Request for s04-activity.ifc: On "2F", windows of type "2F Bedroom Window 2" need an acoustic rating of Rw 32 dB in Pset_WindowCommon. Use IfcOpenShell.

First a look at what the model holds.

```python
import ifcopenshell
import ifcopenshell.util.element

model = ifcopenshell.open("s04-activity.ifc")
print(model.schema)
storey = next(s for s in model.by_type("IfcBuildingStorey") if s.Name == "2F")
windows = [e for e in ifcopenshell.util.element.get_decomposition(storey) if e.is_a("IfcWindow")]
seen = {}
for e in windows:
    element_type = ifcopenshell.util.element.get_type(e)
    key = (element_type.Name if element_type != e and element_type else None, ifcopenshell.util.element.get_pset(e, "Pset_WindowCommon", "AcousticRating"))
    seen[key] = seen.get(key, 0) + 1
for (name, value), count in sorted(seen.items(), key=str):
    print(count, "x", name, "|", value)
```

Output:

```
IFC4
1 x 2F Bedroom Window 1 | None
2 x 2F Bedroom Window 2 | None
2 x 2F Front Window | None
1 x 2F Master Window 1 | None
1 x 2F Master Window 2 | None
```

```python
import ifcopenshell
import ifcopenshell.api.pset
import ifcopenshell.util.element

model = ifcopenshell.open("s04-activity.ifc")

storey = next(s for s in model.by_type("IfcBuildingStorey") if s.Name == "2F")
windows = [e for e in ifcopenshell.util.element.get_decomposition(storey) if e.is_a("IfcWindow")]

count = 0
for e in windows:
    element_type = ifcopenshell.util.element.get_type(e)
    if element_type in (None, e) or element_type.Name != "2F Bedroom Window 2":
        continue
    # add_pset returns the element's existing set when there is one.
    pset = ifcopenshell.api.pset.add_pset(model, product=e, name="Pset_WindowCommon")
    ifcopenshell.api.pset.edit_pset(model, pset=pset, properties={"AcousticRating": "Rw 32 dB"})
    count += 1

print(count, "windows updated")

model.write("s04-activity-out.ifc")
```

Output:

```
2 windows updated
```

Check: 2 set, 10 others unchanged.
